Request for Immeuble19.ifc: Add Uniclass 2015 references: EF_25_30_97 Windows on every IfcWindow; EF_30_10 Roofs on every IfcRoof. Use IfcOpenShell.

First a look at what the model holds.

```python
import ifcopenshell

model = ifcopenshell.open("Immeuble19.ifc")
print(model.schema)
print("classifications:", [c.Name for c in model.by_type("IfcClassification")])
for ifc_class in ("IfcDoor", "IfcRoof", "IfcStair", "IfcWall", "IfcWindow"):
    print(ifc_class, len(model.by_type(ifc_class)))
```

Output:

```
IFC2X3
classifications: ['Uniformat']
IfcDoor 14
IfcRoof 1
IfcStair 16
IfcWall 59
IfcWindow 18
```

```python
import ifcopenshell
import ifcopenshell.api.classification

model = ifcopenshell.open("Immeuble19.ifc")

# IFC2X3 requires Source and Edition and has no link from the project to the system.
system = model.create_entity("IfcClassification", Source="NBS", Edition="2015", Name="Uniclass 2015")

codes = {
    "IfcWindow": ("EF_25_30_97", "Windows"),
    "IfcRoof": ("EF_30_10", "Roofs"),
}
for ifc_class, (code, name) in codes.items():
    products = model.by_type(ifc_class)
    ifcopenshell.api.classification.add_reference(
        model, products=products, classification=system, identification=code, name=name
    )
    print(code, len(products))

model.write("Immeuble19-out.ifc")
```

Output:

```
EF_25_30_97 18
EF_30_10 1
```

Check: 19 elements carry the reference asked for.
